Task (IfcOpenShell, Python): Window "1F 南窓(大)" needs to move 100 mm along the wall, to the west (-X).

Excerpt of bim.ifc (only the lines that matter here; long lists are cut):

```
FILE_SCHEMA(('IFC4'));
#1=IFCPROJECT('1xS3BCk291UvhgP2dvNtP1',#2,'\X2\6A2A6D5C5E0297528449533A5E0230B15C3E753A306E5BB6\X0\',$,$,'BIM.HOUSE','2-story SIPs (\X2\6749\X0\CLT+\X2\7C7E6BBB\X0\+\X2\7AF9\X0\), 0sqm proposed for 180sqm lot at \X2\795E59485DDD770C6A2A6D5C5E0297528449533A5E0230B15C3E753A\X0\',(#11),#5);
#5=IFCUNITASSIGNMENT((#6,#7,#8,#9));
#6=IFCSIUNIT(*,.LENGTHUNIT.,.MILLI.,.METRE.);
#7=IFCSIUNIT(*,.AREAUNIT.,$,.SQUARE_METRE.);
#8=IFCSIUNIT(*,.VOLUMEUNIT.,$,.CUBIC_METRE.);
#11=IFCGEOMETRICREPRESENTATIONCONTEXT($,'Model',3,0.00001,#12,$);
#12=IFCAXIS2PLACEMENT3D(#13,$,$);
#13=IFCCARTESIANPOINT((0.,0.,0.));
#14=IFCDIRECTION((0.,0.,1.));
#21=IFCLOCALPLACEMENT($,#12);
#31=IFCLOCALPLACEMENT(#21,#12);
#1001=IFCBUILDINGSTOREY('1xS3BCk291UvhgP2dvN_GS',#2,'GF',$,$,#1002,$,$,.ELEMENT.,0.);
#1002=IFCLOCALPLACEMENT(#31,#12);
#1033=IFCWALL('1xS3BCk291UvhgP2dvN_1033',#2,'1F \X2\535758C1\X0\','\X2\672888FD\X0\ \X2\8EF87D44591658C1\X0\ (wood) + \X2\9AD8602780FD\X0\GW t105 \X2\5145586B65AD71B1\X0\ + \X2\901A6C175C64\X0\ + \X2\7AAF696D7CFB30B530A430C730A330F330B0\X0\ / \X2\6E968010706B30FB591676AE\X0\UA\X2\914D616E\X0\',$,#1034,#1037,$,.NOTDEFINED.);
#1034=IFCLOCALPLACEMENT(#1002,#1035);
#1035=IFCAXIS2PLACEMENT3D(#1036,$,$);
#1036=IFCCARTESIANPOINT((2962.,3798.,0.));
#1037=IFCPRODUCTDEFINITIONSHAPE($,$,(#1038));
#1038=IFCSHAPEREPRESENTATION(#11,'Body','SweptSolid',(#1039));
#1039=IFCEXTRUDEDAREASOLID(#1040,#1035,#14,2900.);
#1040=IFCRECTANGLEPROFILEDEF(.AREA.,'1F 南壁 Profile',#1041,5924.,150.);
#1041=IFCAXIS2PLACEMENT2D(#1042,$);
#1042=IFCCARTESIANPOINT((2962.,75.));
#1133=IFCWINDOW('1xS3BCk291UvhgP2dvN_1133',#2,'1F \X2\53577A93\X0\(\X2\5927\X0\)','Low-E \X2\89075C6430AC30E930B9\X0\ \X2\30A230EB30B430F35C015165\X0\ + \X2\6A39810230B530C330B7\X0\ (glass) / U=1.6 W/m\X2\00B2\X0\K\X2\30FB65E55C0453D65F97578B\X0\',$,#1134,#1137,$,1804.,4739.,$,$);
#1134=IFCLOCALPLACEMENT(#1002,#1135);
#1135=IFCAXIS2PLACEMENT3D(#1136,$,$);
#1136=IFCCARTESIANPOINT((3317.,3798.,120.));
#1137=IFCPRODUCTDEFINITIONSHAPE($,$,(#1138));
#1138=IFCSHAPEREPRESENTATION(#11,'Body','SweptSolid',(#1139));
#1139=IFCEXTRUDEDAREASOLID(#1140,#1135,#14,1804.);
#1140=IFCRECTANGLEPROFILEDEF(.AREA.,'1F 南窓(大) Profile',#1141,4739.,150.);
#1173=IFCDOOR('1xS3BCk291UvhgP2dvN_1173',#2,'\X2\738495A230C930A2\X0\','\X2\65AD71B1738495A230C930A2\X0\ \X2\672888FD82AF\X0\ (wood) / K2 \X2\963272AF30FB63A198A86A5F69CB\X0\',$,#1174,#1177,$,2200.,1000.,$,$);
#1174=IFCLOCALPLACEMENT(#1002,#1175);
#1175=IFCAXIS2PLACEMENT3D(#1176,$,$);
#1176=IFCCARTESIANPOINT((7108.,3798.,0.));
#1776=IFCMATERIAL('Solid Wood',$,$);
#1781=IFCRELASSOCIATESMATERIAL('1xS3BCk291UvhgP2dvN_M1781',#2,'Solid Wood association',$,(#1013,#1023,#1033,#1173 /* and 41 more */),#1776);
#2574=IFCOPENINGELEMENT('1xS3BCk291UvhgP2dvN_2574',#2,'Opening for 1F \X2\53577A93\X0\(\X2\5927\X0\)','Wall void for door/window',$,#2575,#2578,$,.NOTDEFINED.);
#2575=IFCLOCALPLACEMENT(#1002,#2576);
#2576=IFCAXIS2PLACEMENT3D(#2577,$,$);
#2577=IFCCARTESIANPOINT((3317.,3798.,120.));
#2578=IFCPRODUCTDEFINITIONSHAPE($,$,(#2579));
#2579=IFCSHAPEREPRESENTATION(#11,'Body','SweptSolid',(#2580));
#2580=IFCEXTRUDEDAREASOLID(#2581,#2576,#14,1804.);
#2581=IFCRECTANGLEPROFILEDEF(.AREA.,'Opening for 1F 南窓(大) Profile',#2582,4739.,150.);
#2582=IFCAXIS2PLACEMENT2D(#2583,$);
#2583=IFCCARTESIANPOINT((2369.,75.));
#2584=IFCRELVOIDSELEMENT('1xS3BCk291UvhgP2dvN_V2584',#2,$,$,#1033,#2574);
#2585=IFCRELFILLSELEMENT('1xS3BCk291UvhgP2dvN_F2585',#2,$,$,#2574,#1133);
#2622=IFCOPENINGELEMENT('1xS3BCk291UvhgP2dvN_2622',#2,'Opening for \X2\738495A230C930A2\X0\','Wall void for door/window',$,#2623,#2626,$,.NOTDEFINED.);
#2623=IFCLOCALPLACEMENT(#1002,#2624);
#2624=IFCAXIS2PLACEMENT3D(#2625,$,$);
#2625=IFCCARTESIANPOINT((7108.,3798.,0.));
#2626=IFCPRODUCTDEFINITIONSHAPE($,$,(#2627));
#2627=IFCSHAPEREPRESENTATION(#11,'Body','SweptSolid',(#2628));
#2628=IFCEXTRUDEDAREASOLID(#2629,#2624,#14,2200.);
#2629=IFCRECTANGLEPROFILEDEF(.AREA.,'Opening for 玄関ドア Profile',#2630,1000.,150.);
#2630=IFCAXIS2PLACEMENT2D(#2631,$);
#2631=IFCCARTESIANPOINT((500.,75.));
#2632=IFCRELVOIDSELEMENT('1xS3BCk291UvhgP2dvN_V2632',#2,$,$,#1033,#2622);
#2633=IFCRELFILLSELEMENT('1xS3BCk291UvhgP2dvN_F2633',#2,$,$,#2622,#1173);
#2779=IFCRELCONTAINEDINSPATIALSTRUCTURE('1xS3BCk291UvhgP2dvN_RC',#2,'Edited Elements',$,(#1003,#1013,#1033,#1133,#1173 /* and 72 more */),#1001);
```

```python
import ifcopenshell
import ifcopenshell.api.geometry
import ifcopenshell.util.placement

model = ifcopenshell.open("bim.ifc")

window = model.by_guid("1xS3BCk291UvhgP2dvN_1133")
opening = window.FillsVoids[0].RelatingOpeningElement
wall = opening.VoidsElements[0].RelatingBuildingElement

wall_matrix = ifcopenshell.util.placement.get_local_placement(wall.ObjectPlacement)
shift = wall_matrix[:3, 0] * -100.0
before = ifcopenshell.util.placement.get_local_placement(window.ObjectPlacement)[:3, 3].copy()

# The window is not placed relative to its opening, so move both.
for product in (opening, window):
    matrix = ifcopenshell.util.placement.get_local_placement(product.ObjectPlacement)
    matrix[:3, 3] += shift
    ifcopenshell.api.geometry.edit_object_placement(model, product=product, matrix=matrix, is_si=False)

after = ifcopenshell.util.placement.get_local_placement(window.ObjectPlacement)[:3, 3]
print("window moved by", (after - before).round(3) + 0.0)

model.write("bim_updated.ifc")
```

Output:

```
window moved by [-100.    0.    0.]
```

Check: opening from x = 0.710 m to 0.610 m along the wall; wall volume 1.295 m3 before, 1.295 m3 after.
